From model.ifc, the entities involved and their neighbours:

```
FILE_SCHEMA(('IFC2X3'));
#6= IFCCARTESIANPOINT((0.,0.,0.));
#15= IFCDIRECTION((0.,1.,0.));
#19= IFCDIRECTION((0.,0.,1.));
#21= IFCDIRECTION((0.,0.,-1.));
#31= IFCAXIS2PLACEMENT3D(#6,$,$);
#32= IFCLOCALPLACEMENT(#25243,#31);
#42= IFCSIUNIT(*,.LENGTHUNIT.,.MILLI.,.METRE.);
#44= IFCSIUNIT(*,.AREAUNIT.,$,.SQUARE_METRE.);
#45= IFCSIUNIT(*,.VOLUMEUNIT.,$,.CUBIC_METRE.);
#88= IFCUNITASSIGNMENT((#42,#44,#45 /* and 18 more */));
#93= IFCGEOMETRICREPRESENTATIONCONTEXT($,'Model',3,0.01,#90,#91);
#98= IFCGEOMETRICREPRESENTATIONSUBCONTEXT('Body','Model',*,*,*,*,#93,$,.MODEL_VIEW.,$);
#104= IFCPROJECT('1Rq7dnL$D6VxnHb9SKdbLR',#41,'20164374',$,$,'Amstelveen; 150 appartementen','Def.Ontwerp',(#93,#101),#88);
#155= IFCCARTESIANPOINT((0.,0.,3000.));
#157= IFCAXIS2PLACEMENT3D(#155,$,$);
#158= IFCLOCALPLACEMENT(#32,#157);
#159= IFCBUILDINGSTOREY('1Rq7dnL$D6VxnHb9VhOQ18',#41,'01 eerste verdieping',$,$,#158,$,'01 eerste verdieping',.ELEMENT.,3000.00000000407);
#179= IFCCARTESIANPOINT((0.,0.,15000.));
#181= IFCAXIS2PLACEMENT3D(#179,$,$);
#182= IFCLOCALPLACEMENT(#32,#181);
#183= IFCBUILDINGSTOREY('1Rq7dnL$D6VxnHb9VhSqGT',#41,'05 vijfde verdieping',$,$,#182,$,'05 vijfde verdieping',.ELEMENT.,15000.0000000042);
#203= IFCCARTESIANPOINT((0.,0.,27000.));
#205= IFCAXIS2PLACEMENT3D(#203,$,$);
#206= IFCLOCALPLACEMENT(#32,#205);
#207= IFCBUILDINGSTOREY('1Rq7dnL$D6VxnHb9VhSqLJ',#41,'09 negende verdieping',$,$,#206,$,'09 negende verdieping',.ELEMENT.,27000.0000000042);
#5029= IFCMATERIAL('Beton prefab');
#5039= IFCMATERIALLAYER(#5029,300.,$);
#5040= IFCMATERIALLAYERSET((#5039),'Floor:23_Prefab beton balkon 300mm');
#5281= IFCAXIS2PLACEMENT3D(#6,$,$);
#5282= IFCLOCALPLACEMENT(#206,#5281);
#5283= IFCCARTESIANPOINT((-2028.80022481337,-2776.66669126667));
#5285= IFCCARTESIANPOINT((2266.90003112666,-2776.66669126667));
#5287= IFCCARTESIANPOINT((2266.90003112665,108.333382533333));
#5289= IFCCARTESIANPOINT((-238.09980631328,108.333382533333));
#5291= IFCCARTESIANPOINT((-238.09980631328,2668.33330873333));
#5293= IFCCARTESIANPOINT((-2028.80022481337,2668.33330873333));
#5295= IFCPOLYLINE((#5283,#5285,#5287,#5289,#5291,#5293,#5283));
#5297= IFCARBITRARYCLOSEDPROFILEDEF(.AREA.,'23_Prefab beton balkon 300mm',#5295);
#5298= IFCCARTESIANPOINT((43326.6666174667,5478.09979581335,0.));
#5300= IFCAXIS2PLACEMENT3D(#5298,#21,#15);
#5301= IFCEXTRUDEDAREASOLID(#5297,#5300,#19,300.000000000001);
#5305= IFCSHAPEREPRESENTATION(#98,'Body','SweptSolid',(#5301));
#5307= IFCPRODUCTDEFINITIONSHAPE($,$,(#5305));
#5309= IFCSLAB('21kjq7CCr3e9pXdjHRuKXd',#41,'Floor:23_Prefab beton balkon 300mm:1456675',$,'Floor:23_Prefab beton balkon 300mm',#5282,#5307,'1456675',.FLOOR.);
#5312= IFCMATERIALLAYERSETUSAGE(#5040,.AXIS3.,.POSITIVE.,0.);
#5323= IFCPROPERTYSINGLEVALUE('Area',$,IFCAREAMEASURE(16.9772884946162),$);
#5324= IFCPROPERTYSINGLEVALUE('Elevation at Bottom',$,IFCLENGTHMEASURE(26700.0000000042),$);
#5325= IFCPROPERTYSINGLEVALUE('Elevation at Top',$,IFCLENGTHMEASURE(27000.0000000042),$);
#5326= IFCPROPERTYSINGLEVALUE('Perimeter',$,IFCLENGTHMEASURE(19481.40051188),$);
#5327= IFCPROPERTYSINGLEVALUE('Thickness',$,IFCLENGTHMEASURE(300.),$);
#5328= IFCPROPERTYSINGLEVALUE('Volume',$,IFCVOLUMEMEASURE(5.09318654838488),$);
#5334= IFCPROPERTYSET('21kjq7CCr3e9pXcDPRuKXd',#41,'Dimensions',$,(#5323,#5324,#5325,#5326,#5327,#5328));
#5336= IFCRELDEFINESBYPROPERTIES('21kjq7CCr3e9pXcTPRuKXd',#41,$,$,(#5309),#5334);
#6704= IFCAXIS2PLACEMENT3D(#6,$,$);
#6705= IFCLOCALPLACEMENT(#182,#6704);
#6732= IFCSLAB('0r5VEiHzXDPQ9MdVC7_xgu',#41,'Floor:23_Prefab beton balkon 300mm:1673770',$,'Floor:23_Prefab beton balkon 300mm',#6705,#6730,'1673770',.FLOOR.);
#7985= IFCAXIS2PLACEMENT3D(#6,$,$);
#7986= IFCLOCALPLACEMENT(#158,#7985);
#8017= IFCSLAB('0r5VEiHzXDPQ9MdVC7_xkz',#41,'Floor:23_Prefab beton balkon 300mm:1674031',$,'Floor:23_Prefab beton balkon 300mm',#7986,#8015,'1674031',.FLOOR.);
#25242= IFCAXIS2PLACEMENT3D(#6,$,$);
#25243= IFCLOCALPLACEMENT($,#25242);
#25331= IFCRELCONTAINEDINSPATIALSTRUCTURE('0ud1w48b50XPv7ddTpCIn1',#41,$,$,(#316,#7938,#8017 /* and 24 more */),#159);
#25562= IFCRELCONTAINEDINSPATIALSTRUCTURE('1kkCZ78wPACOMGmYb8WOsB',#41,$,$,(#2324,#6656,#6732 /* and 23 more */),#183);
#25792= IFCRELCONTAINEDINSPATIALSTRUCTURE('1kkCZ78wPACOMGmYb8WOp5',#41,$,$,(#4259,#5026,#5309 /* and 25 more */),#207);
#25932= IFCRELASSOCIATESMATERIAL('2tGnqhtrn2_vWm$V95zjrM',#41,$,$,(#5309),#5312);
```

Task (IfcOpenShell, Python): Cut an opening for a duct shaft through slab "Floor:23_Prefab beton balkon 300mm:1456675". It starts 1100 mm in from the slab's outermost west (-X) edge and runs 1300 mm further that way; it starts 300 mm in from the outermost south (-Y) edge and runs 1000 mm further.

```python
import numpy as np
import ifcopenshell
import ifcopenshell.api.feature
import ifcopenshell.api.geometry
import ifcopenshell.api.pset
import ifcopenshell.api.root
import ifcopenshell.geom
import ifcopenshell.util.element
import ifcopenshell.util.placement
import ifcopenshell.util.representation
import ifcopenshell.util.shape
import ifcopenshell.util.unit

model = ifcopenshell.open("model.ifc")
unit_scale = ifcopenshell.util.unit.calculate_unit_scale(model)
area_scale = ifcopenshell.util.unit.calculate_unit_scale(model, "AREAUNIT")
volume_scale = ifcopenshell.util.unit.calculate_unit_scale(model, "VOLUMEUNIT")
settings = ifcopenshell.geom.settings()


def volume(element):
    """Net volume in cubic metres, openings subtracted."""
    shape = ifcopenshell.geom.create_shape(settings, element)
    return ifcopenshell.util.shape.get_volume(shape.geometry)


slab = model.by_guid("21kjq7CCr3e9pXdjHRuKXd")
before = volume(slab)

# Extent in the slab's own axes, in metres. The edges named are its -X and -Y sides.
slab_shape = ifcopenshell.geom.create_shape(settings, slab)
vertices = ifcopenshell.util.shape.get_vertices(slab_shape.geometry)
x_min, y_min, bottom = vertices.min(axis=0)
top = vertices[:, 2].max()

opening = ifcopenshell.api.root.create_entity(model, ifc_class="IfcOpeningElement", name="Duct shaft opening")
context = ifcopenshell.util.representation.get_context(model, "Model", "Body", "MODEL_VIEW")
width, depth = 1.3, 1
outline = [(0.0, 0.0), (width, 0.0), (width, depth), (0.0, depth), (0.0, 0.0)]
# Overshoot both faces by 50 mm so the cut is clean.
shape = ifcopenshell.api.geometry.add_slab_representation(
    model, context=context, depth=top - bottom + 0.1, polyline=outline
)
ifcopenshell.api.geometry.assign_representation(model, product=opening, representation=shape)

matrix = ifcopenshell.util.placement.get_local_placement(slab.ObjectPlacement)
matrix[:, 3] = matrix @ np.append(np.array([x_min + 1.1, y_min + 0.3, bottom - 0.05]) / unit_scale, 1.0)
ifcopenshell.api.geometry.edit_object_placement(model, product=opening, matrix=matrix, is_si=False)
ifcopenshell.api.feature.add_feature(model, feature=opening, element=slab)

after = volume(slab)

# Update the slab's stored quantities.
pset = model.by_id(ifcopenshell.util.element.get_pset(slab, "Dimensions", should_inherit=False)["id"])
ifcopenshell.api.pset.edit_pset(model, pset=pset, properties={
    "Area": model.create_entity("IfcAreaMeasure", after / (top - bottom) / area_scale),
    "Volume": model.create_entity("IfcVolumeMeasure", after / volume_scale),
})

print(f"slab volume {before:.3f} -> {after:.3f} m3")

model.write("model_updated.ifc")
```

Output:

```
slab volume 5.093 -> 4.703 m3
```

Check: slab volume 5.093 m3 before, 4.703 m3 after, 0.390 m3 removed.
